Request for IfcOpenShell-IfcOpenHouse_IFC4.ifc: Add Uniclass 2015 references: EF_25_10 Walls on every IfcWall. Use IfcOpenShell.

First a look at what the model holds.

```python
import ifcopenshell

model = ifcopenshell.open("IfcOpenShell-IfcOpenHouse_IFC4.ifc")
print(model.schema)
print("classifications:", [c.Name for c in model.by_type("IfcClassification")])
for ifc_class in ("IfcDoor", "IfcRoof", "IfcStair", "IfcWall", "IfcWindow"):
    print(ifc_class, len(model.by_type(ifc_class)))
```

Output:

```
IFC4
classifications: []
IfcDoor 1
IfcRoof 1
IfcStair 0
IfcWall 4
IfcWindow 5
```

```python
import ifcopenshell
import ifcopenshell.api.classification

model = ifcopenshell.open("IfcOpenShell-IfcOpenHouse_IFC4.ifc")

system = ifcopenshell.api.classification.add_classification(model, classification="Uniclass 2015")

codes = {
    "IfcWall": ("EF_25_10", "Walls"),
}
for ifc_class, (code, name) in codes.items():
    products = model.by_type(ifc_class)
    ifcopenshell.api.classification.add_reference(
        model, products=products, classification=system, identification=code, name=name
    )
    print(code, len(products))

model.write("IfcOpenShell-IfcOpenHouse_IFC4-out.ifc")
```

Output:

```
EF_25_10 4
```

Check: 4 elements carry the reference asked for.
